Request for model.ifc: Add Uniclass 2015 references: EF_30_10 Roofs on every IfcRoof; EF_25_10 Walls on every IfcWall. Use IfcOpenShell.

First a look at what the model holds.

```python
import ifcopenshell

model = ifcopenshell.open("model.ifc")
print(model.schema)
print("classifications:", [c.Name for c in model.by_type("IfcClassification")])
for ifc_class in ("IfcDoor", "IfcRoof", "IfcStair", "IfcWall", "IfcWindow"):
    print(ifc_class, len(model.by_type(ifc_class)))
```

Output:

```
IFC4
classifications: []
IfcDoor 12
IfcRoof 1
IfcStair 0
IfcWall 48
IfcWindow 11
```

```python
import ifcopenshell
import ifcopenshell.api.classification

model = ifcopenshell.open("model.ifc")

system = ifcopenshell.api.classification.add_classification(model, classification="Uniclass 2015")

codes = {
    "IfcRoof": ("EF_30_10", "Roofs"),
    "IfcWall": ("EF_25_10", "Walls"),
}
for ifc_class, (code, name) in codes.items():
    products = model.by_type(ifc_class)
    ifcopenshell.api.classification.add_reference(
        model, products=products, classification=system, identification=code, name=name
    )
    print(code, len(products))

model.write("model_rev.ifc")
```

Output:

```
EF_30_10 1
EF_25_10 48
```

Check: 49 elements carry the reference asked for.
